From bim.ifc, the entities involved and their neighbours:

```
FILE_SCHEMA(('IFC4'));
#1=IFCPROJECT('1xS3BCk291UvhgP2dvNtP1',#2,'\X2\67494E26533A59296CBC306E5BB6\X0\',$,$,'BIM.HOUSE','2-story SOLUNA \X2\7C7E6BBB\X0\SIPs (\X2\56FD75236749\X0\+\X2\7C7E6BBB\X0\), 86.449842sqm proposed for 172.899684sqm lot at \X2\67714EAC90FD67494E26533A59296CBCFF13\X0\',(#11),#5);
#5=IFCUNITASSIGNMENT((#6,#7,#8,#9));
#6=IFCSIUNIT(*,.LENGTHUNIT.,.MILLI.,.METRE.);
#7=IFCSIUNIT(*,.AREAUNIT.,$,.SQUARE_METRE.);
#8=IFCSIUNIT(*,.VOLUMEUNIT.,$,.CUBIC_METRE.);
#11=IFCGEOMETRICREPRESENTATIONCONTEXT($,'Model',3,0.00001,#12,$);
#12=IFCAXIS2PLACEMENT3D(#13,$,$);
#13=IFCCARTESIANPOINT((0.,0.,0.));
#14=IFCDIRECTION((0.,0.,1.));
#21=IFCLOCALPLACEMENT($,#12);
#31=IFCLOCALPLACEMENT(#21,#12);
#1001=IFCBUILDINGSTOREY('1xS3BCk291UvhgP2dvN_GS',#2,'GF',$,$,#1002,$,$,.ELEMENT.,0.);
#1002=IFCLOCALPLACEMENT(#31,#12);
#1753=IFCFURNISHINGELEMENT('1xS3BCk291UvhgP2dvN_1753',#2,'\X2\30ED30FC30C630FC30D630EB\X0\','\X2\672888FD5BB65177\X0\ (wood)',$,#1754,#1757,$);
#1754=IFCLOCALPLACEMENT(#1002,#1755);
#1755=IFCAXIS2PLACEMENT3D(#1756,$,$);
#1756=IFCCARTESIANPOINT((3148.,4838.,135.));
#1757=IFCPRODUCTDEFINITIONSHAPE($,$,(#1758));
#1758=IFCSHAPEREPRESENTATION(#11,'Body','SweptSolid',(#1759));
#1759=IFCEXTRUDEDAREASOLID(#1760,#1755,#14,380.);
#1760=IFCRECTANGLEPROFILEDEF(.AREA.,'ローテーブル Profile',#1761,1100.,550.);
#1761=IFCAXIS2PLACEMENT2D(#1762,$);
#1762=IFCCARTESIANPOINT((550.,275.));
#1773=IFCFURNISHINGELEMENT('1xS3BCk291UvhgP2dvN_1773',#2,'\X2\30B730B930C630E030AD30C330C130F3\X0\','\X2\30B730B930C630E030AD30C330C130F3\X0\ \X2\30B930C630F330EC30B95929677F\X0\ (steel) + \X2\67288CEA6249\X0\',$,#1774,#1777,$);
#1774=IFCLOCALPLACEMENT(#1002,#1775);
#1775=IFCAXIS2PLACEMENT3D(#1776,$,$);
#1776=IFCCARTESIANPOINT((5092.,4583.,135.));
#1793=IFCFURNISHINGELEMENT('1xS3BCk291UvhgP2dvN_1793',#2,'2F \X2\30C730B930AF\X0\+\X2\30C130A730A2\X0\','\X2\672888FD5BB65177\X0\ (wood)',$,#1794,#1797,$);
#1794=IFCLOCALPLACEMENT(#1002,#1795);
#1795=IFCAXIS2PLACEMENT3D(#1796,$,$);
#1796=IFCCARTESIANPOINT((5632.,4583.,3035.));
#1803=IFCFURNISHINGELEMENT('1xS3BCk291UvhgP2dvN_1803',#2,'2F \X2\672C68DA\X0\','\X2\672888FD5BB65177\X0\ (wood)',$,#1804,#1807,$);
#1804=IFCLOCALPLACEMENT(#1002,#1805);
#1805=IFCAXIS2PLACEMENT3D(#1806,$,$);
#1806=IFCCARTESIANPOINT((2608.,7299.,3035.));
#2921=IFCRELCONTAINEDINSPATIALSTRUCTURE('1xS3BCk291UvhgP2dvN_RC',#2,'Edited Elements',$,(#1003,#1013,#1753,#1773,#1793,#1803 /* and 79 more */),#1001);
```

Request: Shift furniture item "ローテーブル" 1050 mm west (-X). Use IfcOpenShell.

```python
import ifcopenshell
import ifcopenshell.api.geometry
import ifcopenshell.util.placement

model = ifcopenshell.open("bim.ifc")

item = model.by_guid("1xS3BCk291UvhgP2dvN_1753")
matrix = ifcopenshell.util.placement.get_local_placement(item.ObjectPlacement)
matrix[0, 3] -= 1050.0
ifcopenshell.api.geometry.edit_object_placement(model, product=item, matrix=matrix, is_si=False)

print(ifcopenshell.util.placement.get_local_placement(item.ObjectPlacement).round(3) + 0.0)

model.write("bim_rev.ifc")
```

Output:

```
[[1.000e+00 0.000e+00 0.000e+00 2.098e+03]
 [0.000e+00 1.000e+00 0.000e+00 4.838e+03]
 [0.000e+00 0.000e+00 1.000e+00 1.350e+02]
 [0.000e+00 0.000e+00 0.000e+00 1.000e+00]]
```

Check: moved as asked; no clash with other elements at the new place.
